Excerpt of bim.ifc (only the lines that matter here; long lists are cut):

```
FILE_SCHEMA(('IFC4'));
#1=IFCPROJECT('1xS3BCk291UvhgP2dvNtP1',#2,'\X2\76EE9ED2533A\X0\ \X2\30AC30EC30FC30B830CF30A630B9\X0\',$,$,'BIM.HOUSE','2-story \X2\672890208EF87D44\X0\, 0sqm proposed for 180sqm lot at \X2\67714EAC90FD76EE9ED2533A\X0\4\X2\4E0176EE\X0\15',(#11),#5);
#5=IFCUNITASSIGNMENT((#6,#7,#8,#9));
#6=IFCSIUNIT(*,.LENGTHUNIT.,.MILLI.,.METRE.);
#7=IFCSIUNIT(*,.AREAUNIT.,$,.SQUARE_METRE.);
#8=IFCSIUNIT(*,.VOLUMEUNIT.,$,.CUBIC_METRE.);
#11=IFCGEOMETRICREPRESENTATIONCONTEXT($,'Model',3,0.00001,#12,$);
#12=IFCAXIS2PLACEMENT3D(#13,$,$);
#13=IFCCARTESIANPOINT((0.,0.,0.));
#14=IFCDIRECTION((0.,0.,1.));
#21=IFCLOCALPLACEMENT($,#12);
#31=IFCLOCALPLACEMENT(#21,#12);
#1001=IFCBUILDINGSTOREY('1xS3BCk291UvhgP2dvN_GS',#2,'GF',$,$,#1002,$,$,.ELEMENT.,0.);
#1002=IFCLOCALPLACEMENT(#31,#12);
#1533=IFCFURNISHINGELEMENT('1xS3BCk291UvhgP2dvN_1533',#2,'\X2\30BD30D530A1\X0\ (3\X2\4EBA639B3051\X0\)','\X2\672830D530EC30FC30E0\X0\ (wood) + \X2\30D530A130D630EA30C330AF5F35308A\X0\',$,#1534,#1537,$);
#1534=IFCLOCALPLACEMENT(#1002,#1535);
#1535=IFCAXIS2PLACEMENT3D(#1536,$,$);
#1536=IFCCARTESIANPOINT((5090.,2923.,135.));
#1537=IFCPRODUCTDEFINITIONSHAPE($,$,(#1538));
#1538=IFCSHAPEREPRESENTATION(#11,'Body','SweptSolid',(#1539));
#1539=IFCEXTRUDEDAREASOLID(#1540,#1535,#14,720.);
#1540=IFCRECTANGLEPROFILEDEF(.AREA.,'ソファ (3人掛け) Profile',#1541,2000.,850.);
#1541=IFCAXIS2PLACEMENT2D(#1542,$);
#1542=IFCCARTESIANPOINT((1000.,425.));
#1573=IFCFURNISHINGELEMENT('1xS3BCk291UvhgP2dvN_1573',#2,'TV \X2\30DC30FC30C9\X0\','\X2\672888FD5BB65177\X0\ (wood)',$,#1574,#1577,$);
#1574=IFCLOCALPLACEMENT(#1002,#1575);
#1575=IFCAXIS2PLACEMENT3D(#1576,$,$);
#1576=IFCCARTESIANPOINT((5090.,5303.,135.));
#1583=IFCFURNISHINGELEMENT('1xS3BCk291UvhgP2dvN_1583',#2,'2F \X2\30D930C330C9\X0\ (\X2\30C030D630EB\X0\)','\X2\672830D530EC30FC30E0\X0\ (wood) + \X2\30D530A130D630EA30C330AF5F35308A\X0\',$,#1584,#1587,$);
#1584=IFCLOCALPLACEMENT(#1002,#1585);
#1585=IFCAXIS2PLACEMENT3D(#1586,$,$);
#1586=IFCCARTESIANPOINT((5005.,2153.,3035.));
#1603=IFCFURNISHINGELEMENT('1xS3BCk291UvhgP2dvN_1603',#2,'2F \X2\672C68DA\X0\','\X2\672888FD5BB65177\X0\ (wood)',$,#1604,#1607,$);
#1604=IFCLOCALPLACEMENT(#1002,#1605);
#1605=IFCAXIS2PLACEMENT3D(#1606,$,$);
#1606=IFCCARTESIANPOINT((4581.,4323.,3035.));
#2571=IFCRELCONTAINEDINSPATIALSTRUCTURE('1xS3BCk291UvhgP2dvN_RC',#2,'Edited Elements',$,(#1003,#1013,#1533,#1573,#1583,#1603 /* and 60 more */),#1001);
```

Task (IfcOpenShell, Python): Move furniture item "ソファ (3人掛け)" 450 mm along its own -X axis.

```python
import ifcopenshell
import ifcopenshell.api.geometry
import ifcopenshell.util.placement
import ifcopenshell.util.unit

model = ifcopenshell.open("bim.ifc")
unit_scale = ifcopenshell.util.unit.calculate_unit_scale(model)

item = model.by_guid("1xS3BCk291UvhgP2dvN_1533")
matrix = ifcopenshell.util.placement.get_local_placement(item.ObjectPlacement)
matrix[:3, 3] -= matrix[:3, 0] * 0.45 / unit_scale
ifcopenshell.api.geometry.edit_object_placement(model, product=item, matrix=matrix, is_si=False)

print(ifcopenshell.util.placement.get_local_placement(item.ObjectPlacement).round(3) + 0.0)

model.write("bim_rev.ifc")
```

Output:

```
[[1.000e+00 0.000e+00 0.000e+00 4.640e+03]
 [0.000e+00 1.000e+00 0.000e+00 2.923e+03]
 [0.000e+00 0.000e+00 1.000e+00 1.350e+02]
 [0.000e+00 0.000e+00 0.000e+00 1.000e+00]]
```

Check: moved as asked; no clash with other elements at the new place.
